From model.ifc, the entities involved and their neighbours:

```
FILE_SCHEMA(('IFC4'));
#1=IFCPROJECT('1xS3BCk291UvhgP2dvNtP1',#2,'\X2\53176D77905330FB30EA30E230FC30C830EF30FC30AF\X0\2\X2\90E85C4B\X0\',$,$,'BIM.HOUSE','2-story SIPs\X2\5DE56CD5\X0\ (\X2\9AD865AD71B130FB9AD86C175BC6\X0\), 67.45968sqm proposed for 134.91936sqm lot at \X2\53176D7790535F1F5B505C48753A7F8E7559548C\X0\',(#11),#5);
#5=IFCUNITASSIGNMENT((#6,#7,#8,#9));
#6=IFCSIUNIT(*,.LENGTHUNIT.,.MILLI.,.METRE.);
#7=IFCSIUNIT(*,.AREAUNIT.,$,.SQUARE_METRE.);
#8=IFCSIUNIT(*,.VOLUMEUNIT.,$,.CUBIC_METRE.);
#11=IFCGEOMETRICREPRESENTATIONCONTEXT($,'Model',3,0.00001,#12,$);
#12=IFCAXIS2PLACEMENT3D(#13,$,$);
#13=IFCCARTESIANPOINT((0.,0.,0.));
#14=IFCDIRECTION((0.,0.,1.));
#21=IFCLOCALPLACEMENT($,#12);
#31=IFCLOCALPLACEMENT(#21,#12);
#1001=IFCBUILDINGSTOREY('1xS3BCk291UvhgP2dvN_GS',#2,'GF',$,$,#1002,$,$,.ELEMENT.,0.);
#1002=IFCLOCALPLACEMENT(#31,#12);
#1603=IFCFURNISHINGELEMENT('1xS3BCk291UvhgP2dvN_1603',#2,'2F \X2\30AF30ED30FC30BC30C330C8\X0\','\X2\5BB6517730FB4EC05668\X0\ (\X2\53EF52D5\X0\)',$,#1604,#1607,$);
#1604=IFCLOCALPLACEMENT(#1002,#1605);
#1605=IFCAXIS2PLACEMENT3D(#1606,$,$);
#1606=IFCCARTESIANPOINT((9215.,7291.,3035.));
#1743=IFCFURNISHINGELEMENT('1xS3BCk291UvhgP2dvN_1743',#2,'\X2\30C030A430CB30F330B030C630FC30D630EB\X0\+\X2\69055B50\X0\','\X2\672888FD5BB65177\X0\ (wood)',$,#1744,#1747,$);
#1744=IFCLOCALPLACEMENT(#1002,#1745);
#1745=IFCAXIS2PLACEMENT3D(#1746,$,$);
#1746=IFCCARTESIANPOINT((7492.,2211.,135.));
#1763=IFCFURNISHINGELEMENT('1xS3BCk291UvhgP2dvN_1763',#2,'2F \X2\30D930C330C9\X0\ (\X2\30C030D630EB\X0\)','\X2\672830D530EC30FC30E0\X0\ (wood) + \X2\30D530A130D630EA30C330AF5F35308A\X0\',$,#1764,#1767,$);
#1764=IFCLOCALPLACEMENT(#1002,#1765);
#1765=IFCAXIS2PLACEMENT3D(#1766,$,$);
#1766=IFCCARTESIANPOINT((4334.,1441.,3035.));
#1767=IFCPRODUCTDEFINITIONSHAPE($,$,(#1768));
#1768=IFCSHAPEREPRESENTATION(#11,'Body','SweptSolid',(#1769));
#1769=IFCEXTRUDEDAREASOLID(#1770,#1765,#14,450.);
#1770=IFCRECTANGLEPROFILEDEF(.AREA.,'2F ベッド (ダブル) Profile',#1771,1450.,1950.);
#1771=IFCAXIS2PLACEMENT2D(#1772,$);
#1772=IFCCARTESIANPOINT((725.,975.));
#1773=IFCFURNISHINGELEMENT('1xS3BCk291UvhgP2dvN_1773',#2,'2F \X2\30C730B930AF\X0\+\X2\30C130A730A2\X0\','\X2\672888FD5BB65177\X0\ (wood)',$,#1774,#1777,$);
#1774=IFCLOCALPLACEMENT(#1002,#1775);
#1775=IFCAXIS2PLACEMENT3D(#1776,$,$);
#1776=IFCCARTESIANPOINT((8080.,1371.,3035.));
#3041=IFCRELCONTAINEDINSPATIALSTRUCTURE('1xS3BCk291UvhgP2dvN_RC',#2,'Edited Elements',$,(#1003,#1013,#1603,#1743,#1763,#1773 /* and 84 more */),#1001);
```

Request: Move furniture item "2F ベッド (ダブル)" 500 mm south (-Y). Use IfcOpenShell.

```python
import ifcopenshell
import ifcopenshell.api.geometry
import ifcopenshell.util.placement
import ifcopenshell.util.unit

model = ifcopenshell.open("model.ifc")
unit_scale = ifcopenshell.util.unit.calculate_unit_scale(model)

item = model.by_guid("1xS3BCk291UvhgP2dvN_1763")
matrix = ifcopenshell.util.placement.get_local_placement(item.ObjectPlacement)
matrix[1, 3] -= 0.5 / unit_scale
ifcopenshell.api.geometry.edit_object_placement(model, product=item, matrix=matrix, is_si=False)

print(ifcopenshell.util.placement.get_local_placement(item.ObjectPlacement).round(3) + 0.0)

model.write("model_edited.ifc")
```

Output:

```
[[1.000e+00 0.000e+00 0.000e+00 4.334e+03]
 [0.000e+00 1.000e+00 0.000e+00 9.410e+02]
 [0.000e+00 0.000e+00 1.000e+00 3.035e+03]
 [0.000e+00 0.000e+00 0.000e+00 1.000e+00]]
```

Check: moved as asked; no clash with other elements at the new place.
